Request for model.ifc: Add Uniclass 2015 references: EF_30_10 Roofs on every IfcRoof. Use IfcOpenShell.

First a look at what the model holds.

```python
import ifcopenshell

model = ifcopenshell.open("model.ifc")
print(model.schema)
print("classifications:", [c.Name for c in model.by_type("IfcClassification")])
for ifc_class in ("IfcDoor", "IfcRoof", "IfcStair", "IfcWall", "IfcWindow"):
    print(ifc_class, len(model.by_type(ifc_class)))
```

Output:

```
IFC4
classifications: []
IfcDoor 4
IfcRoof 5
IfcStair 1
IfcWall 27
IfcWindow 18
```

```python
import ifcopenshell
import ifcopenshell.api.classification

model = ifcopenshell.open("model.ifc")

system = ifcopenshell.api.classification.add_classification(model, classification="Uniclass 2015")

codes = {
    "IfcRoof": ("EF_30_10", "Roofs"),
}
for ifc_class, (code, name) in codes.items():
    products = model.by_type(ifc_class)
    ifcopenshell.api.classification.add_reference(
        model, products=products, classification=system, identification=code, name=name
    )
    print(code, len(products))

model.write("model_v2.ifc")
```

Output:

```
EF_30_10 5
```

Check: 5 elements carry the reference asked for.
